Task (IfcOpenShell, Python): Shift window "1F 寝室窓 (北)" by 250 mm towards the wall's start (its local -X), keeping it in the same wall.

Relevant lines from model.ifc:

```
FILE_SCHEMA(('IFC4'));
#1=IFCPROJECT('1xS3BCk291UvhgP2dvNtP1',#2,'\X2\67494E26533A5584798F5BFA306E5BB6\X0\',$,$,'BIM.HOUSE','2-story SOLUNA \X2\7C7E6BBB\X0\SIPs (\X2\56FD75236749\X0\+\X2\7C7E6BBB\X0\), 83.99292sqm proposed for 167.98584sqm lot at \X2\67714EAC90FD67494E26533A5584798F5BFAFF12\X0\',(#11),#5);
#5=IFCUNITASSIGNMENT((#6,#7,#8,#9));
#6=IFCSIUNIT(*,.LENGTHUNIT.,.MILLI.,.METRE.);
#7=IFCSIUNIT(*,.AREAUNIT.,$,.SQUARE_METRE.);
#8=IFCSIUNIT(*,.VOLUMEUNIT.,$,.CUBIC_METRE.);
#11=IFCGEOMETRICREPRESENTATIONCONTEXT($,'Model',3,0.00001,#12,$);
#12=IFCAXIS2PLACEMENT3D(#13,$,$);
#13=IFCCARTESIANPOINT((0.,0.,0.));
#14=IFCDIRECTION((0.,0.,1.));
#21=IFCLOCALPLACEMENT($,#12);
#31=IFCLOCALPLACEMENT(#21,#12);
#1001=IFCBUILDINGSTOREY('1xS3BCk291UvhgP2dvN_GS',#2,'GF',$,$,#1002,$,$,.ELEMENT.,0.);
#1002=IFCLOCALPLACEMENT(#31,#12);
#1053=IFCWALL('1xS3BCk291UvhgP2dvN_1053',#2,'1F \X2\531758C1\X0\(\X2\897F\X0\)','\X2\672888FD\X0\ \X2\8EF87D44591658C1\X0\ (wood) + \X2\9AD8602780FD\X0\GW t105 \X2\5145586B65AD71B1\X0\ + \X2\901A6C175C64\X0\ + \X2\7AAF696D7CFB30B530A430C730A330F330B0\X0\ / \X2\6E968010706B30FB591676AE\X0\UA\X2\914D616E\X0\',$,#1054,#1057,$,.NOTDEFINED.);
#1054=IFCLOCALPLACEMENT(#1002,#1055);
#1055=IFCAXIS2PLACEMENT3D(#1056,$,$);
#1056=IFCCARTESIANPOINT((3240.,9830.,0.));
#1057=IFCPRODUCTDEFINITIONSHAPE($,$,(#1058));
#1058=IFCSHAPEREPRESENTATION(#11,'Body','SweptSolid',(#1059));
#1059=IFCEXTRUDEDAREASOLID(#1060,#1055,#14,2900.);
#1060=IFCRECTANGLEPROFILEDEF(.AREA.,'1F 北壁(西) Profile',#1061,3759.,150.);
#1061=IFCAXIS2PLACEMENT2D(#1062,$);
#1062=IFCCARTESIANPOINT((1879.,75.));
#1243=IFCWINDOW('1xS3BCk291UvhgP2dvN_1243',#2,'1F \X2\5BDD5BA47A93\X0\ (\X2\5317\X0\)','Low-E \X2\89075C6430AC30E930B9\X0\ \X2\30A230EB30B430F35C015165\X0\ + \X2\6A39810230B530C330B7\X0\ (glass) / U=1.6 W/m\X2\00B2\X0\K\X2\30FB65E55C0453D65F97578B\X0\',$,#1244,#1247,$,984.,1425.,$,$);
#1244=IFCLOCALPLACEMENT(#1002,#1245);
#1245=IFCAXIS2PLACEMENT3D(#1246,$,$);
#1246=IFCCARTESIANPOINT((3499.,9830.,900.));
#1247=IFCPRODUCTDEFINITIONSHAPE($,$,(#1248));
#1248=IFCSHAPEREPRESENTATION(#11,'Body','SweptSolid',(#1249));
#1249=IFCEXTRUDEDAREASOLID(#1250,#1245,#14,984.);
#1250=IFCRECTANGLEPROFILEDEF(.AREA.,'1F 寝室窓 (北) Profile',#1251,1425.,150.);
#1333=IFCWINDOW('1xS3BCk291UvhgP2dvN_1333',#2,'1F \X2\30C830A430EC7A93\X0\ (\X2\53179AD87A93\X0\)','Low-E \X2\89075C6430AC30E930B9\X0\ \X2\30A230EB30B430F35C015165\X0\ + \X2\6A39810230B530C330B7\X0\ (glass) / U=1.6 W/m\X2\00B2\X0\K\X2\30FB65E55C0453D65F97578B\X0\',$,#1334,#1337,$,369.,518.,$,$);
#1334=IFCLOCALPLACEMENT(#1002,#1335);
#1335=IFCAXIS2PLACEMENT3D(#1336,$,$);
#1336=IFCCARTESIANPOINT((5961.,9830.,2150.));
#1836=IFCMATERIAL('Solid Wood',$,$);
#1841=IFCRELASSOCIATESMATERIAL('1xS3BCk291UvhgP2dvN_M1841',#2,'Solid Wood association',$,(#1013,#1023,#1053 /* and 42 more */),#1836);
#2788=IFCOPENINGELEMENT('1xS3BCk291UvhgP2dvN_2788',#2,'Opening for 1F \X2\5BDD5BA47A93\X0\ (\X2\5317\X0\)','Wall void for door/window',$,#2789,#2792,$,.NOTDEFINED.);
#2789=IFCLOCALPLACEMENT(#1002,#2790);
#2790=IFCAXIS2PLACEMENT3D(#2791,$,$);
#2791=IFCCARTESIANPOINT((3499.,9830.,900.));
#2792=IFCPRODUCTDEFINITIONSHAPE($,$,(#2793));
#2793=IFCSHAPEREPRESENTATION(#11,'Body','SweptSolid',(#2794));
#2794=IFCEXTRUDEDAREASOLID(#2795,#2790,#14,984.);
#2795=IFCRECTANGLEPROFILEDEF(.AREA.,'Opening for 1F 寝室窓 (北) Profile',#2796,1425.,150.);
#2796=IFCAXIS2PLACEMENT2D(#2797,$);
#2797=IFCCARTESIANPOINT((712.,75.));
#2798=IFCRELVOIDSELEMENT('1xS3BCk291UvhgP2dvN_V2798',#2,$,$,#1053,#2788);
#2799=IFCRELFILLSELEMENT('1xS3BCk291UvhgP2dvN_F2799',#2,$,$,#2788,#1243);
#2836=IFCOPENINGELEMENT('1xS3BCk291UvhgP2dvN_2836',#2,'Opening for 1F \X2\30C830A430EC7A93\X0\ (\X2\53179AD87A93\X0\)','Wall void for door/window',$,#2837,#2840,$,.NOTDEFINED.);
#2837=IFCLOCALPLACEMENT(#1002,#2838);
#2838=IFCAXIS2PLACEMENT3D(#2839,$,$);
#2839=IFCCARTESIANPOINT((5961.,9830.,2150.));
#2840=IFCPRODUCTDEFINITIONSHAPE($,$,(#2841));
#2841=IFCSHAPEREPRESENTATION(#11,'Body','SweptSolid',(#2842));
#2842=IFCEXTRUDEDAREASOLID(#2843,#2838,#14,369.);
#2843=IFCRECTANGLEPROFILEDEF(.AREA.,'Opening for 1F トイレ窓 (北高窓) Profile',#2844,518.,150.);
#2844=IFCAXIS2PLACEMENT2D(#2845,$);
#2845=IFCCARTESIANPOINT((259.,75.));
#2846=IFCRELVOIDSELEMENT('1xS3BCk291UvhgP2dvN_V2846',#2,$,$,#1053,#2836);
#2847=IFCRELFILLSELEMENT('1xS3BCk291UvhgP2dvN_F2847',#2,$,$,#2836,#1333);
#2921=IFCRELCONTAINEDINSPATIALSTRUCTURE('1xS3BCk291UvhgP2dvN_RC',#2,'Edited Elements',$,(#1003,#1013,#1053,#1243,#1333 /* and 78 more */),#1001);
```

```python
import ifcopenshell
import ifcopenshell.api.geometry
import ifcopenshell.util.placement
import ifcopenshell.util.unit

model = ifcopenshell.open("model.ifc")
unit_scale = ifcopenshell.util.unit.calculate_unit_scale(model)

window = model.by_id(1243)
opening = window.FillsVoids[0].RelatingOpeningElement
wall = opening.VoidsElements[0].RelatingBuildingElement

wall_matrix = ifcopenshell.util.placement.get_local_placement(wall.ObjectPlacement)
shift = wall_matrix[:3, 0] * -0.25 / unit_scale
before = ifcopenshell.util.placement.get_local_placement(window.ObjectPlacement)[:3, 3].copy()

# The window is not placed relative to its opening, so move both.
for product in (opening, window):
    matrix = ifcopenshell.util.placement.get_local_placement(product.ObjectPlacement)
    matrix[:3, 3] += shift
    ifcopenshell.api.geometry.edit_object_placement(model, product=product, matrix=matrix, is_si=False)

after = ifcopenshell.util.placement.get_local_placement(window.ObjectPlacement)[:3, 3]
print("window moved by", (after - before).round(3) + 0.0)

model.write("model_rev.ifc")
```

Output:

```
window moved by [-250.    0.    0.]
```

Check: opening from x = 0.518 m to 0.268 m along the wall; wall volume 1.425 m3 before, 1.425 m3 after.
